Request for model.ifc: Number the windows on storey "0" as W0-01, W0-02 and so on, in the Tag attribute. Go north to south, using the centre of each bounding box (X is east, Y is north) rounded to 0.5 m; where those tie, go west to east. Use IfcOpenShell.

First a look at what the model holds.

```python
import ifcopenshell
import ifcopenshell.util.element
import ifcopenshell.util.placement

model = ifcopenshell.open("model.ifc")
print(model.schema)
storey = next(s for s in model.by_type("IfcBuildingStorey") if s.Name == "0")
windows = [e for e in ifcopenshell.util.element.get_decomposition(storey) if e.is_a("IfcWindow")]
for e in sorted(windows, key=lambda e: e.id()):
    origin = ifcopenshell.util.placement.get_local_placement(e.ObjectPlacement)[:3, 3]
    print(e.id(), e.Tag, e.Name, origin.round(2) + 0.0, sep=" | ")
```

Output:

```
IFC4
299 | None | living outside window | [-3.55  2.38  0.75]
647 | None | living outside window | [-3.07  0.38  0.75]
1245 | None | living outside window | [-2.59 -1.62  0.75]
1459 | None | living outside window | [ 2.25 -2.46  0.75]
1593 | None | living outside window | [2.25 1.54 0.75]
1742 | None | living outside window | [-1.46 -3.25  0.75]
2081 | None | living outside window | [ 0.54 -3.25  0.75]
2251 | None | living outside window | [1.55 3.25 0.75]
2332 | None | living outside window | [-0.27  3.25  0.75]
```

```python
import ifcopenshell
import ifcopenshell.geom
import ifcopenshell.util.element
import ifcopenshell.util.shape

model = ifcopenshell.open("model.ifc")
settings = ifcopenshell.geom.settings()
settings.set("use-world-coords", True)


def centre(element):
    shape = ifcopenshell.geom.create_shape(settings, element)
    return ifcopenshell.util.shape.get_bbox_centroid(shape.geometry)


storey = next(s for s in model.by_type("IfcBuildingStorey") if s.Name == "0")
windows = [e for e in ifcopenshell.util.element.get_decomposition(storey) if e.is_a("IfcWindow")]

# Insertion points can sit at a corner or the storey origin, so sort by the geometry (in metres).
centres = {e: centre(e) for e in windows}
windows.sort(key=lambda e: (-round(centres[e][1] / 0.5), centres[e][0]))

for i, e in enumerate(windows, start=1):
    number = f"W0-{i:02d}"
    e.Tag = number
    print(e.id(), number)

model.write("model_edited.ifc")
```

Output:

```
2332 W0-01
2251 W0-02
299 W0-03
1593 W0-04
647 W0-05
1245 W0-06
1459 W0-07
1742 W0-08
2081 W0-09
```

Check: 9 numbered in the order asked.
